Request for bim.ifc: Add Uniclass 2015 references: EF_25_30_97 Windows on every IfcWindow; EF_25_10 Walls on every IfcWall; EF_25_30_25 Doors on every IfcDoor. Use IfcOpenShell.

First a look at what the model holds.

```python
import ifcopenshell

model = ifcopenshell.open("bim.ifc")
print(model.schema)
print("classifications:", [c.Name for c in model.by_type("IfcClassification")])
for ifc_class in ("IfcDoor", "IfcRoof", "IfcStair", "IfcWall", "IfcWindow"):
    print(ifc_class, len(model.by_type(ifc_class)))
```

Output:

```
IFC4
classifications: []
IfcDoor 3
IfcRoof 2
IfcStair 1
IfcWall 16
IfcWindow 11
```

```python
import ifcopenshell
import ifcopenshell.api.classification

model = ifcopenshell.open("bim.ifc")

system = ifcopenshell.api.classification.add_classification(model, classification="Uniclass 2015")

codes = {
    "IfcWindow": ("EF_25_30_97", "Windows"),
    "IfcWall": ("EF_25_10", "Walls"),
    "IfcDoor": ("EF_25_30_25", "Doors"),
}
for ifc_class, (code, name) in codes.items():
    products = model.by_type(ifc_class)
    ifcopenshell.api.classification.add_reference(
        model, products=products, classification=system, identification=code, name=name
    )
    print(code, len(products))

model.write("bim_rev.ifc")
```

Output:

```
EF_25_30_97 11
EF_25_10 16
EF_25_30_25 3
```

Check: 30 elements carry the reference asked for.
